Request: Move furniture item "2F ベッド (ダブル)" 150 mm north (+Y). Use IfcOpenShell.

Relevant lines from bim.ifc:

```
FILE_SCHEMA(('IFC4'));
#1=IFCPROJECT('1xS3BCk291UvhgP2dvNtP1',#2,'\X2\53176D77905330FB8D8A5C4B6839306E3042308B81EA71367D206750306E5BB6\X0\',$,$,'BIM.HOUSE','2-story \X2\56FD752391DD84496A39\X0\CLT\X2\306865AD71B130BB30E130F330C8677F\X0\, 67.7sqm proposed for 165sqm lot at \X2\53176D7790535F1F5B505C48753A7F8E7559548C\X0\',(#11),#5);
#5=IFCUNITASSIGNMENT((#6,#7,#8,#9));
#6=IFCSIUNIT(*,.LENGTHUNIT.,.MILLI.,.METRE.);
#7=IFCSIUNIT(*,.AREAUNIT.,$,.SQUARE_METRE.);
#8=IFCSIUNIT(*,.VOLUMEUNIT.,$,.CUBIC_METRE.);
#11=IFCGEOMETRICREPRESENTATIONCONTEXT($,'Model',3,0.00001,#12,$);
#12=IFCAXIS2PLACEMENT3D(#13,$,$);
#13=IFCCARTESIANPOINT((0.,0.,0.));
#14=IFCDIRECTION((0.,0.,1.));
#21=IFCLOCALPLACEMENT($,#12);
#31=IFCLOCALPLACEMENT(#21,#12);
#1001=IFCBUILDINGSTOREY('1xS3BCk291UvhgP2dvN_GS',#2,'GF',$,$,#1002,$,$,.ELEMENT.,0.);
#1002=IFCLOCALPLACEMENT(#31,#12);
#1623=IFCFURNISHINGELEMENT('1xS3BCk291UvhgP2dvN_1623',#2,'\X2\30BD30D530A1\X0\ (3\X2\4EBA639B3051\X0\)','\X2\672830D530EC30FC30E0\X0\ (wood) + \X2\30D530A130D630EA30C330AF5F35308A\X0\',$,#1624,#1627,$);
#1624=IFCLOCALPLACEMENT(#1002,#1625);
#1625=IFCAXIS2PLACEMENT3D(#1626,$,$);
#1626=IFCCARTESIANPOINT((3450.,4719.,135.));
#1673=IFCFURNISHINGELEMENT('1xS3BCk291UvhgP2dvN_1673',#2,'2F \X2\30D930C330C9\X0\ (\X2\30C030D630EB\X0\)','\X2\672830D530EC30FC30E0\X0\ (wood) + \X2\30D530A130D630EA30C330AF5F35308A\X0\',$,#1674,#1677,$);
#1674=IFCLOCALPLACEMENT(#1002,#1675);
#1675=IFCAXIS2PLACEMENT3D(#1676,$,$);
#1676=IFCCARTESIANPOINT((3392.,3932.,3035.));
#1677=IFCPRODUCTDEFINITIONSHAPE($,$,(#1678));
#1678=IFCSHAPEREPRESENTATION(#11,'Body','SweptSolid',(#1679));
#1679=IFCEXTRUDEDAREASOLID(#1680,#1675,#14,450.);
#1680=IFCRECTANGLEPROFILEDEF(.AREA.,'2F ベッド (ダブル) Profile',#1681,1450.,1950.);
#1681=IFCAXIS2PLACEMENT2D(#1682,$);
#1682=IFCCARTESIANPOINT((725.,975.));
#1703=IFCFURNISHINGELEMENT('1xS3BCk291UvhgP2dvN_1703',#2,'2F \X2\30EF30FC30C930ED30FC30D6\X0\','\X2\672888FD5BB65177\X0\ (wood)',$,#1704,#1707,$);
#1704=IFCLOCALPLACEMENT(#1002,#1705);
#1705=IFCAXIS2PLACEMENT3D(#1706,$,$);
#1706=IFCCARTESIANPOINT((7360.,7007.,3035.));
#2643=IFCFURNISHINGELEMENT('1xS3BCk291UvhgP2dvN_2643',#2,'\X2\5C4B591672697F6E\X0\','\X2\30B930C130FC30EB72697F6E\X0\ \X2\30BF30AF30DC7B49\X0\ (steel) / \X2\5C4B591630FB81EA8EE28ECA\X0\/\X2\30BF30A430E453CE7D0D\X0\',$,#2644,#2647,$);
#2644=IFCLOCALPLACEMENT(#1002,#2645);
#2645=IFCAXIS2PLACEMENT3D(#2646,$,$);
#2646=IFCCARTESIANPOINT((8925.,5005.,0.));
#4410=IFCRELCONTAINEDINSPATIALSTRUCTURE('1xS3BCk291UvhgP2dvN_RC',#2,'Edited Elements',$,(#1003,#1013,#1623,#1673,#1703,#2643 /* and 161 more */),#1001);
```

```python
import ifcopenshell
import ifcopenshell.api.geometry
import ifcopenshell.util.placement

model = ifcopenshell.open("bim.ifc")

item = model.by_id(1673)
matrix = ifcopenshell.util.placement.get_local_placement(item.ObjectPlacement)
matrix[1, 3] += 150.0
ifcopenshell.api.geometry.edit_object_placement(model, product=item, matrix=matrix, is_si=False)

print(ifcopenshell.util.placement.get_local_placement(item.ObjectPlacement).round(3) + 0.0)

model.write("bim_v2.ifc")
```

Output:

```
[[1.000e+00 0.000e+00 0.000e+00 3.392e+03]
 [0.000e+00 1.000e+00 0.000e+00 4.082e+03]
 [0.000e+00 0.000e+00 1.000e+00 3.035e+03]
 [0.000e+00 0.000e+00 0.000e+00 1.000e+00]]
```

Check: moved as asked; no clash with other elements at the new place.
